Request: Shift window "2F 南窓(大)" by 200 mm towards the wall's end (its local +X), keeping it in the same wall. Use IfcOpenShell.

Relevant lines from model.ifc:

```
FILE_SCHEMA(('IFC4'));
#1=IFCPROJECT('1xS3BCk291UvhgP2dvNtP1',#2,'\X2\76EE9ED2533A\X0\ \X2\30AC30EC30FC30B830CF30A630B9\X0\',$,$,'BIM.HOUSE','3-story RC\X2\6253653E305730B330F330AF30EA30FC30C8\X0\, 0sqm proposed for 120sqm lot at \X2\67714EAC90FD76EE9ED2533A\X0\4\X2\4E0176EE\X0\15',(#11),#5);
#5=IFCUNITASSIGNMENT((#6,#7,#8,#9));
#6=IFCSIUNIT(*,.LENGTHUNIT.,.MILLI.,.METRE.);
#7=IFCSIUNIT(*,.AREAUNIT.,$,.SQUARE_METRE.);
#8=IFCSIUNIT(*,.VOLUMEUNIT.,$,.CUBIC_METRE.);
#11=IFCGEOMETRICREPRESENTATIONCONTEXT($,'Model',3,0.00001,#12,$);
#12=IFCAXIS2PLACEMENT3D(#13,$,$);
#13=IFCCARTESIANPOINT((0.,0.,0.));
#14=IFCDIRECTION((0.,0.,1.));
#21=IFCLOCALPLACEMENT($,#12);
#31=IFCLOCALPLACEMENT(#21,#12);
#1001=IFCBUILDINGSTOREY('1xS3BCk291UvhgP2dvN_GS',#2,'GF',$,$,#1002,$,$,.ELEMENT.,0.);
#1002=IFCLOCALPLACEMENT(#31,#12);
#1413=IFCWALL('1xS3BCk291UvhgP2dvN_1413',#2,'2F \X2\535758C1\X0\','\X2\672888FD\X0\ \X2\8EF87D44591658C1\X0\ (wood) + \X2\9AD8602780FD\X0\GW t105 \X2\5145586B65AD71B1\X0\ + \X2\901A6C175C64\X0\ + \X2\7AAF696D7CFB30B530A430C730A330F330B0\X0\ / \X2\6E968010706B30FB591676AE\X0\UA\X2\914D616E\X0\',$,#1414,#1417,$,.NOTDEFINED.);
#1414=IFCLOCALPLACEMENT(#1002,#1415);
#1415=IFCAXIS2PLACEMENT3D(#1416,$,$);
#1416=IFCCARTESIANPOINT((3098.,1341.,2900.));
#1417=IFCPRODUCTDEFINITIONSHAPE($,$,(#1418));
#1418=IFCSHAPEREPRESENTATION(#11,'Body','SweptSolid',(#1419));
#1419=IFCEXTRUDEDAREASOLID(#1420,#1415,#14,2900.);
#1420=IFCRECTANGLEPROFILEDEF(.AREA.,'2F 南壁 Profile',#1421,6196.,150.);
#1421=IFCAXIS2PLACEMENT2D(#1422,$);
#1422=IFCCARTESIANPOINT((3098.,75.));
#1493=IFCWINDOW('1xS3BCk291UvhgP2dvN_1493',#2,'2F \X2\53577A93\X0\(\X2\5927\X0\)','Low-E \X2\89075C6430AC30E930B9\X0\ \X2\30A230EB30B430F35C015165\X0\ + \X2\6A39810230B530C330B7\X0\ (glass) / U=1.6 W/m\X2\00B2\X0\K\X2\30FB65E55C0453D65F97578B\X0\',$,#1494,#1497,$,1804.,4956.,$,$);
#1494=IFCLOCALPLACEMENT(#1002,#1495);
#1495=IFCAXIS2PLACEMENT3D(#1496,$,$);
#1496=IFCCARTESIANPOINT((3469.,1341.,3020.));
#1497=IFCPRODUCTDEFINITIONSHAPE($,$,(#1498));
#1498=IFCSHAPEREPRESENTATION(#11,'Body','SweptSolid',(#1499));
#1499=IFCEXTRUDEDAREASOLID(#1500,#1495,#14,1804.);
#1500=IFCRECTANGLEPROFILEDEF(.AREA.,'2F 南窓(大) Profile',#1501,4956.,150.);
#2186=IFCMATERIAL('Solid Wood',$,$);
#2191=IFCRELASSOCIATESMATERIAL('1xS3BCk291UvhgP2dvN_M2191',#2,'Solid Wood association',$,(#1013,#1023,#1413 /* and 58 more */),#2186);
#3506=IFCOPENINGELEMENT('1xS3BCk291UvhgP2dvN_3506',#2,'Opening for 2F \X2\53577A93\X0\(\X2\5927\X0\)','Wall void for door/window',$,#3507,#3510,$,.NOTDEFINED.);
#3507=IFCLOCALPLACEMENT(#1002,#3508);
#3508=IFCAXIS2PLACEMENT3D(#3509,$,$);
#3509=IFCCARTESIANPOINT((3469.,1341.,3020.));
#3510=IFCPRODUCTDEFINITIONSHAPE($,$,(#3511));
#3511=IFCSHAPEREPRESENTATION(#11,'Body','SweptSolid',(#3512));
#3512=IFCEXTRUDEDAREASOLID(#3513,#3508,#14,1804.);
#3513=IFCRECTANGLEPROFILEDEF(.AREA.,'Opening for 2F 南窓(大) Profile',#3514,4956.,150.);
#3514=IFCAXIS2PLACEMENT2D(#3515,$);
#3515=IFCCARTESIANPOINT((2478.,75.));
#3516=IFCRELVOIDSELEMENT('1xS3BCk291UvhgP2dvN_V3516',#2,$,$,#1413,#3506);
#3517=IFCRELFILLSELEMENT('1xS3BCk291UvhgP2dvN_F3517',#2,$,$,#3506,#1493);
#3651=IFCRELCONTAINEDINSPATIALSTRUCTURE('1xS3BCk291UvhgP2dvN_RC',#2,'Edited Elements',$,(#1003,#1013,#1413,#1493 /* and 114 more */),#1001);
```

```python
import ifcopenshell
import ifcopenshell.api.geometry
import ifcopenshell.util.placement
import ifcopenshell.util.unit

model = ifcopenshell.open("model.ifc")
unit_scale = ifcopenshell.util.unit.calculate_unit_scale(model)

window = model.by_guid("1xS3BCk291UvhgP2dvN_1493")
opening = window.FillsVoids[0].RelatingOpeningElement
wall = opening.VoidsElements[0].RelatingBuildingElement

wall_matrix = ifcopenshell.util.placement.get_local_placement(wall.ObjectPlacement)
shift = wall_matrix[:3, 0] * 0.2 / unit_scale
before = ifcopenshell.util.placement.get_local_placement(window.ObjectPlacement)[:3, 3].copy()

# The window is not placed relative to its opening, so move both.
for product in (opening, window):
    matrix = ifcopenshell.util.placement.get_local_placement(product.ObjectPlacement)
    matrix[:3, 3] += shift
    ifcopenshell.api.geometry.edit_object_placement(model, product=product, matrix=matrix, is_si=False)

after = ifcopenshell.util.placement.get_local_placement(window.ObjectPlacement)[:3, 3]
print("window moved by", (after - before).round(3) + 0.0)

model.write("model_v2.ifc")
```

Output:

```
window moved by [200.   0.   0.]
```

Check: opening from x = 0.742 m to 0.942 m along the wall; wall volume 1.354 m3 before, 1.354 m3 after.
